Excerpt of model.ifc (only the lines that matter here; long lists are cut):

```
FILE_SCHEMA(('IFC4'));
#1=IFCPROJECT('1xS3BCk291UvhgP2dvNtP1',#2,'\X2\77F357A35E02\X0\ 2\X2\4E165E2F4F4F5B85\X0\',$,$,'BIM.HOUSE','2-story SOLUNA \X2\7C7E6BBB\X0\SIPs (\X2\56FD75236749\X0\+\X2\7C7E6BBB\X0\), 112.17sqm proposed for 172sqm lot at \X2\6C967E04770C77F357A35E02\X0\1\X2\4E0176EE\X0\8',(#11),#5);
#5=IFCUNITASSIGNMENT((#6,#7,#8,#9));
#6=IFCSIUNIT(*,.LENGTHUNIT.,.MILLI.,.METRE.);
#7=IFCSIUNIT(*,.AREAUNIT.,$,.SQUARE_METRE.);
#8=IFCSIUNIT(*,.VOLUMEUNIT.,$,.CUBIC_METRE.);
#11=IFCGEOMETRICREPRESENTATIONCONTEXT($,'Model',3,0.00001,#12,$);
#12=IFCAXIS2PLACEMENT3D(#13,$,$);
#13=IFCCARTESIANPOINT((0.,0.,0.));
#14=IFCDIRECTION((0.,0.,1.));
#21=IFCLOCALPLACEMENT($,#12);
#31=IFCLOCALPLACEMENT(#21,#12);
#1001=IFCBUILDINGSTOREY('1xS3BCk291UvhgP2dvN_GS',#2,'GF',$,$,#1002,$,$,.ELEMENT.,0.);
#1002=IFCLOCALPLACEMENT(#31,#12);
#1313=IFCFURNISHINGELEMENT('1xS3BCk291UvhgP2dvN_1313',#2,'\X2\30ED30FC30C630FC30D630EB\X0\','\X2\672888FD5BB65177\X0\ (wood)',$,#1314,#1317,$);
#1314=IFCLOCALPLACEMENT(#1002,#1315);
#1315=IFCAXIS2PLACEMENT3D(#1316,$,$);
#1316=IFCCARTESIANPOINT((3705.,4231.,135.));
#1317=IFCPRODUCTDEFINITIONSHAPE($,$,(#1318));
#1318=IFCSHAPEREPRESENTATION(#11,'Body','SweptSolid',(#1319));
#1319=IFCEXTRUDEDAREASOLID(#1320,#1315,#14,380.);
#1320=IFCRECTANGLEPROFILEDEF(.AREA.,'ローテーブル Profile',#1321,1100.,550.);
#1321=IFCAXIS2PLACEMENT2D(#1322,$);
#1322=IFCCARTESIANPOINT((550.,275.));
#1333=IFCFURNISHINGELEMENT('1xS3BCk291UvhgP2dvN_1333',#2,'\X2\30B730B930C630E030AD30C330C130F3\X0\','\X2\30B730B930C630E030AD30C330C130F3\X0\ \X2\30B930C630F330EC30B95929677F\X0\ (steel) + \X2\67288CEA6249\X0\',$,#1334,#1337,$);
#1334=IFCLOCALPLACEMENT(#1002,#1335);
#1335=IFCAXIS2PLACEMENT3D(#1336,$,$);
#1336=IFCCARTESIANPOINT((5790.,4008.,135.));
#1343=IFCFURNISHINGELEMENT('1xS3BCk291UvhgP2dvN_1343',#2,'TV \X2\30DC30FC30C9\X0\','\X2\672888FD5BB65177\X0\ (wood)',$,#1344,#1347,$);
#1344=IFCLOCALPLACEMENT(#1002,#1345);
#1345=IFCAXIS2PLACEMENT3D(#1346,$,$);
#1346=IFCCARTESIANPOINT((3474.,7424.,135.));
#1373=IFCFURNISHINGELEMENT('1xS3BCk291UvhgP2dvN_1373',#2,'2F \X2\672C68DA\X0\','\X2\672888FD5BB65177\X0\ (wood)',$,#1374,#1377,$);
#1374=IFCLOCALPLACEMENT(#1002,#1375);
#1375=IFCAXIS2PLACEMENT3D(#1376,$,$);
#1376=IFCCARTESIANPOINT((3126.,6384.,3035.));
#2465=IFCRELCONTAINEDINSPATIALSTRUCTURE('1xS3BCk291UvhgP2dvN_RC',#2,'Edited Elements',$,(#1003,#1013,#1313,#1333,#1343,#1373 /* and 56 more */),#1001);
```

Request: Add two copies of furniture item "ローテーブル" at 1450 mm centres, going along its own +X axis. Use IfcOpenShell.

```python
import ifcopenshell
import ifcopenshell.api.geometry
import ifcopenshell.api.root
import ifcopenshell.util.element
import ifcopenshell.util.placement

model = ifcopenshell.open("model.ifc")


def reuse_history(source, copy):
    """copy_class also copies each property set's owner history, people and application; keep the originals."""
    for rel in copy.IsDefinedBy:
        if rel.is_a("IfcRelDefinesByProperties") and (history := rel.RelatingPropertyDefinition.OwnerHistory):
            rel.RelatingPropertyDefinition.OwnerHistory = source.OwnerHistory
            ifcopenshell.util.element.remove_deep2(model, history)


source = model.by_guid("1xS3BCk291UvhgP2dvN_1313")
base = ifcopenshell.util.placement.get_local_placement(source.ObjectPlacement)
step = base[:3, 0] * 1450.0

for i in range(1, 3):
    copy = ifcopenshell.api.root.copy_class(model, product=source)
    copy.Representation = ifcopenshell.util.element.copy_deep(
        model, source.Representation, exclude=["IfcGeometricRepresentationContext", "IfcRepresentationMap"]
    )
    reuse_history(source, copy)
    matrix = base.copy()
    matrix[:3, 3] += i * step
    print("added at", matrix[:3, 3].round(3) + 0.0)
    ifcopenshell.api.geometry.edit_object_placement(model, product=copy, matrix=matrix, is_si=False)

model.write("model_rev.ifc")
```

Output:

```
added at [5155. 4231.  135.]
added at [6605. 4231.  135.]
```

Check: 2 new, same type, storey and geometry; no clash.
